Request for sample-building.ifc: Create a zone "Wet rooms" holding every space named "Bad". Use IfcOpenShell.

First a look at what the model holds.

```python
import ifcopenshell

model = ifcopenshell.open("sample-building.ifc")
print(model.schema)
seen = {}
for space in model.by_type("IfcSpace"):
    seen[space.LongName] = seen.get(space.LongName, 0) + 1
for name, count in sorted(seen.items(), key=str):
    print(count, "x", name)
print("zones:", [z.Name for z in model.by_type("IfcZone")][:20])
```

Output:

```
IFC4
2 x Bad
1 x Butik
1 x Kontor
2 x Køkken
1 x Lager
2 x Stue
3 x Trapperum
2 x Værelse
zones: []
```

```python
import ifcopenshell
import ifcopenshell.api.group
import ifcopenshell.api.root

model = ifcopenshell.open("sample-building.ifc")

names = {"Bad"}
spaces = [s for s in model.by_type("IfcSpace") if s.LongName in names]

zone = ifcopenshell.api.root.create_entity(model, ifc_class="IfcZone", name="Wet rooms")
ifcopenshell.api.group.assign_group(model, products=spaces, group=zone)
print(len(spaces), "spaces in", zone.Name)

model.write("sample-building_v2.ifc")
```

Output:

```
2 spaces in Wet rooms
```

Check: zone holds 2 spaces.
